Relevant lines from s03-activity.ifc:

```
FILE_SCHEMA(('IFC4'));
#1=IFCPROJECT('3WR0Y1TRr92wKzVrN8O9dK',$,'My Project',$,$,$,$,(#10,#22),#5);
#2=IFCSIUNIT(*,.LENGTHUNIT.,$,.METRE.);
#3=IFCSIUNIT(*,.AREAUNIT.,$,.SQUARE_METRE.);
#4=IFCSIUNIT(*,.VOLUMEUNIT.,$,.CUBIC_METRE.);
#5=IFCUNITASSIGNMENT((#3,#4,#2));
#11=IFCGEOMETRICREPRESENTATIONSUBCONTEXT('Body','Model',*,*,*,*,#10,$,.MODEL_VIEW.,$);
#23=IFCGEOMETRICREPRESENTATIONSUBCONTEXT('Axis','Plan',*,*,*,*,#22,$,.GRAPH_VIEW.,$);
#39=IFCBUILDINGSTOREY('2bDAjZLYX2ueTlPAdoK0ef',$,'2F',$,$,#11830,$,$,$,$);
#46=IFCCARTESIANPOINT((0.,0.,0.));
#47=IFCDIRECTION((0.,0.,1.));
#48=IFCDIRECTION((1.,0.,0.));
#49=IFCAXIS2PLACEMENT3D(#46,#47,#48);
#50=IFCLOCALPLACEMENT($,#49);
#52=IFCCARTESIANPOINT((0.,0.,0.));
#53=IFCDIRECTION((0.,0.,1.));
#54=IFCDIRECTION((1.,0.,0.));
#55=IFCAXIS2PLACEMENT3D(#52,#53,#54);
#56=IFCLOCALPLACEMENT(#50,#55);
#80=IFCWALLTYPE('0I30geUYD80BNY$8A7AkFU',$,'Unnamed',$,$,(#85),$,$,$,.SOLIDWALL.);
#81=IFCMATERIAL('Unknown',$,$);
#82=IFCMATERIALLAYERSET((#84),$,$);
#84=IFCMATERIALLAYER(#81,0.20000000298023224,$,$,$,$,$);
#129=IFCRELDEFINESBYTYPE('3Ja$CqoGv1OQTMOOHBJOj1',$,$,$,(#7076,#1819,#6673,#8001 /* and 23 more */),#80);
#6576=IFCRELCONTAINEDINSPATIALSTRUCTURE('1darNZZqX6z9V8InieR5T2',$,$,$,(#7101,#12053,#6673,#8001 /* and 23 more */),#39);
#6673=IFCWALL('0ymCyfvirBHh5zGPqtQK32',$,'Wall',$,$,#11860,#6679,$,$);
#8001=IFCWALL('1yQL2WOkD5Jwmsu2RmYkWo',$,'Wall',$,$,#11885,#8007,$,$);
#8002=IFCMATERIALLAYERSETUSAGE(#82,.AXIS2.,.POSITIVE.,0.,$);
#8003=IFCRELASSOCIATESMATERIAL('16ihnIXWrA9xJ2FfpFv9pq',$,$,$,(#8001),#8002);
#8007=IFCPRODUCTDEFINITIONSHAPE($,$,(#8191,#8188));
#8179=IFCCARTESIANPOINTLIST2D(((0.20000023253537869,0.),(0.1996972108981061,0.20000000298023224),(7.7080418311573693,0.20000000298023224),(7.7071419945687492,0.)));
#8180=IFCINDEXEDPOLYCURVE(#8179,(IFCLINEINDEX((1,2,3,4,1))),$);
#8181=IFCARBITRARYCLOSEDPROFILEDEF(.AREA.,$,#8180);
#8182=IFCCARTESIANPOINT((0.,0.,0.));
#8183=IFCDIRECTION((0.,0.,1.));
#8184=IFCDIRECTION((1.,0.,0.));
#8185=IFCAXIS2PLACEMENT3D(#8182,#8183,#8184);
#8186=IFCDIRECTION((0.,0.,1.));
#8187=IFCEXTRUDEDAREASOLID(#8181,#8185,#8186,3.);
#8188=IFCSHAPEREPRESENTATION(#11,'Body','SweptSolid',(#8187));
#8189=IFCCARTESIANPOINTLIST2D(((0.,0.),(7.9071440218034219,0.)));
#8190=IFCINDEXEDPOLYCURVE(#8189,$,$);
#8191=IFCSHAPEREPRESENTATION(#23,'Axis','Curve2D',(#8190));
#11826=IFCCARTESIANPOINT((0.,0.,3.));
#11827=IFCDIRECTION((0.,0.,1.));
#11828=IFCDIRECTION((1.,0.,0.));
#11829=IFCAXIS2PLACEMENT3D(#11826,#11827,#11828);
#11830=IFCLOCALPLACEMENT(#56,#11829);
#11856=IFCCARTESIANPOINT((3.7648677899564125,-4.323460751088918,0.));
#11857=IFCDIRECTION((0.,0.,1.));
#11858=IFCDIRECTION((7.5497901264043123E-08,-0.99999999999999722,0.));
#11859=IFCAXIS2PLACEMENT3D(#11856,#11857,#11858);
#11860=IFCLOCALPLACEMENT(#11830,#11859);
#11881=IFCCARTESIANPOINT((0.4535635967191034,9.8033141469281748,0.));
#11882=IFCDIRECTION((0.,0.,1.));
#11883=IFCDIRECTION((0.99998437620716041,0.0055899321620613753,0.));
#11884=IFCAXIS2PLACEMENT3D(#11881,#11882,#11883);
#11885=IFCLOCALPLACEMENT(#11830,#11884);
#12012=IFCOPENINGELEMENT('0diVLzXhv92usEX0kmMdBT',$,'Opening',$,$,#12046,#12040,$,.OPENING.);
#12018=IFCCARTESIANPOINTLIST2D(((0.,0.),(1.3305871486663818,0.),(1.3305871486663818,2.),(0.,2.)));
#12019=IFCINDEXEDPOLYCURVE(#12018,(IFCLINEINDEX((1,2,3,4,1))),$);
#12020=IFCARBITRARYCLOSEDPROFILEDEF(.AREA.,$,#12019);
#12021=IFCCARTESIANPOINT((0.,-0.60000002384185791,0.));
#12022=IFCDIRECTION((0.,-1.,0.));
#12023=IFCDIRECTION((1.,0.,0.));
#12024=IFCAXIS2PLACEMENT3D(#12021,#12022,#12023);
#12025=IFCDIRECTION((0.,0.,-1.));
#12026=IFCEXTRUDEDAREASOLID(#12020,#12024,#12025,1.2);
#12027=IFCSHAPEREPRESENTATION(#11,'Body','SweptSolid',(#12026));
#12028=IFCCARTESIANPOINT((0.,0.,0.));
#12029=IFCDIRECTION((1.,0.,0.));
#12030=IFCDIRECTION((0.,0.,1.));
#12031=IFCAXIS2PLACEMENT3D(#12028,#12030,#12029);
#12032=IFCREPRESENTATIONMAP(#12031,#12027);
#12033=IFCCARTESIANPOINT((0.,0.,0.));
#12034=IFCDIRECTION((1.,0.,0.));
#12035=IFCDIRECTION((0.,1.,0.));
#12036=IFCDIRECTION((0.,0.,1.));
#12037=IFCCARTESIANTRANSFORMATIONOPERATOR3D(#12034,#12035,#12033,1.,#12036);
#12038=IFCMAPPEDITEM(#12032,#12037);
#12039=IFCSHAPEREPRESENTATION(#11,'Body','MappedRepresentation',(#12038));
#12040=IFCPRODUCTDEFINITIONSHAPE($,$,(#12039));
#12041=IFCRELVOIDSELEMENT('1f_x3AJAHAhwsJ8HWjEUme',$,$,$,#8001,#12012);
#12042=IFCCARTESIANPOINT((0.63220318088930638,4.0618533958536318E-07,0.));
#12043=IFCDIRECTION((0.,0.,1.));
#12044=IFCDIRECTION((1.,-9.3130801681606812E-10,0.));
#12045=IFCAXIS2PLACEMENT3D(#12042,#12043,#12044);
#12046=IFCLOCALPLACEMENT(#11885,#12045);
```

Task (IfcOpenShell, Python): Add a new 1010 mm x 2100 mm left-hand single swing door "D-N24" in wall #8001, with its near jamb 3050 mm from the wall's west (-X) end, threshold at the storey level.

```python
import numpy as np
import ifcopenshell
import ifcopenshell.api.feature
import ifcopenshell.api.geometry
import ifcopenshell.api.root
import ifcopenshell.api.spatial
import ifcopenshell.geom
import ifcopenshell.util.element
import ifcopenshell.util.placement
import ifcopenshell.util.representation
import ifcopenshell.util.shape
import ifcopenshell.util.unit

model = ifcopenshell.open("s03-activity.ifc")
unit_scale = ifcopenshell.util.unit.calculate_unit_scale(model)
settings = ifcopenshell.geom.settings()


def volume(element):
    """Net volume in cubic metres, openings subtracted."""
    shape = ifcopenshell.geom.create_shape(settings, element)
    return ifcopenshell.util.shape.get_volume(shape.geometry)


wall = model.by_guid("1yQL2WOkD5Jwmsu2RmYkWo")
storey = ifcopenshell.util.element.get_container(wall, ifc_class="IfcBuildingStorey")
context = ifcopenshell.util.representation.get_context(model, "Model", "Body", "MODEL_VIEW")
before = volume(wall)

width, height, from_end, sill = 1.01, 2.1, 3.05, 0.0  # metres

# The wall runs along its own X axis, and the end named is its -X end.
wall_shape = ifcopenshell.geom.create_shape(settings, wall)
x, y, z = ifcopenshell.util.shape.get_vertices(wall_shape.geometry).T
start = x.min() + from_end
face, thickness = float(y.min()), float(y.max() - y.min())
wall_matrix = ifcopenshell.util.placement.get_local_placement(wall.ObjectPlacement)
level = ifcopenshell.util.placement.get_local_placement(storey.ObjectPlacement)[2, 3]


def in_wall(x, y):
    """Placement at x, y metres in the wall's axes, at sill height."""
    matrix = wall_matrix.copy()
    matrix[:, 3] = wall_matrix @ np.array([x / unit_scale, y / unit_scale, 0.0, 1.0])
    matrix[2, 3] = level + sill / unit_scale
    return matrix


# Opening: a box that overshoots both wall faces by 50 mm.
opening = ifcopenshell.api.root.create_entity(model, ifc_class="IfcOpeningElement", predefined_type="OPENING")
box = ifcopenshell.api.geometry.add_wall_representation(
    model, context=context, length=width, height=height, thickness=thickness + 0.1
)
ifcopenshell.api.geometry.assign_representation(model, product=opening, representation=box)
ifcopenshell.api.geometry.edit_object_placement(model, product=opening, matrix=in_wall(start, face - 0.05), is_si=False)
ifcopenshell.api.feature.add_feature(model, feature=opening, element=wall)

door = ifcopenshell.api.root.create_entity(model, ifc_class="IfcDoor", name="D-N24", predefined_type="DOOR")
door.OverallWidth, door.OverallHeight = width / unit_scale, height / unit_scale
door.OperationType = "SINGLE_SWING_LEFT"
body = ifcopenshell.api.geometry.add_door_representation(
    model,
    context=context,
    overall_width=door.OverallWidth,
    overall_height=door.OverallHeight,
    operation_type="SINGLE_SWING_LEFT",
    lining_properties={"LiningDepth": thickness / unit_scale, "ThresholdDepth": thickness / unit_scale},
)
ifcopenshell.api.geometry.assign_representation(model, product=door, representation=body)
ifcopenshell.api.spatial.assign_container(model, products=[door], relating_structure=storey)
ifcopenshell.api.feature.add_filling(model, opening=opening, element=door)

# The lining spans the wall, so the door starts at the wall face.
ifcopenshell.api.geometry.edit_object_placement(model, product=door, matrix=in_wall(start, face), is_si=False)

after = volume(wall)

print(f"wall volume {before:.3f} -> {after:.3f} m3")

model.write("s03-activity_edited.ifc")
```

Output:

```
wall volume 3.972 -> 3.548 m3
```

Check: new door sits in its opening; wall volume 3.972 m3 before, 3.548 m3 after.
